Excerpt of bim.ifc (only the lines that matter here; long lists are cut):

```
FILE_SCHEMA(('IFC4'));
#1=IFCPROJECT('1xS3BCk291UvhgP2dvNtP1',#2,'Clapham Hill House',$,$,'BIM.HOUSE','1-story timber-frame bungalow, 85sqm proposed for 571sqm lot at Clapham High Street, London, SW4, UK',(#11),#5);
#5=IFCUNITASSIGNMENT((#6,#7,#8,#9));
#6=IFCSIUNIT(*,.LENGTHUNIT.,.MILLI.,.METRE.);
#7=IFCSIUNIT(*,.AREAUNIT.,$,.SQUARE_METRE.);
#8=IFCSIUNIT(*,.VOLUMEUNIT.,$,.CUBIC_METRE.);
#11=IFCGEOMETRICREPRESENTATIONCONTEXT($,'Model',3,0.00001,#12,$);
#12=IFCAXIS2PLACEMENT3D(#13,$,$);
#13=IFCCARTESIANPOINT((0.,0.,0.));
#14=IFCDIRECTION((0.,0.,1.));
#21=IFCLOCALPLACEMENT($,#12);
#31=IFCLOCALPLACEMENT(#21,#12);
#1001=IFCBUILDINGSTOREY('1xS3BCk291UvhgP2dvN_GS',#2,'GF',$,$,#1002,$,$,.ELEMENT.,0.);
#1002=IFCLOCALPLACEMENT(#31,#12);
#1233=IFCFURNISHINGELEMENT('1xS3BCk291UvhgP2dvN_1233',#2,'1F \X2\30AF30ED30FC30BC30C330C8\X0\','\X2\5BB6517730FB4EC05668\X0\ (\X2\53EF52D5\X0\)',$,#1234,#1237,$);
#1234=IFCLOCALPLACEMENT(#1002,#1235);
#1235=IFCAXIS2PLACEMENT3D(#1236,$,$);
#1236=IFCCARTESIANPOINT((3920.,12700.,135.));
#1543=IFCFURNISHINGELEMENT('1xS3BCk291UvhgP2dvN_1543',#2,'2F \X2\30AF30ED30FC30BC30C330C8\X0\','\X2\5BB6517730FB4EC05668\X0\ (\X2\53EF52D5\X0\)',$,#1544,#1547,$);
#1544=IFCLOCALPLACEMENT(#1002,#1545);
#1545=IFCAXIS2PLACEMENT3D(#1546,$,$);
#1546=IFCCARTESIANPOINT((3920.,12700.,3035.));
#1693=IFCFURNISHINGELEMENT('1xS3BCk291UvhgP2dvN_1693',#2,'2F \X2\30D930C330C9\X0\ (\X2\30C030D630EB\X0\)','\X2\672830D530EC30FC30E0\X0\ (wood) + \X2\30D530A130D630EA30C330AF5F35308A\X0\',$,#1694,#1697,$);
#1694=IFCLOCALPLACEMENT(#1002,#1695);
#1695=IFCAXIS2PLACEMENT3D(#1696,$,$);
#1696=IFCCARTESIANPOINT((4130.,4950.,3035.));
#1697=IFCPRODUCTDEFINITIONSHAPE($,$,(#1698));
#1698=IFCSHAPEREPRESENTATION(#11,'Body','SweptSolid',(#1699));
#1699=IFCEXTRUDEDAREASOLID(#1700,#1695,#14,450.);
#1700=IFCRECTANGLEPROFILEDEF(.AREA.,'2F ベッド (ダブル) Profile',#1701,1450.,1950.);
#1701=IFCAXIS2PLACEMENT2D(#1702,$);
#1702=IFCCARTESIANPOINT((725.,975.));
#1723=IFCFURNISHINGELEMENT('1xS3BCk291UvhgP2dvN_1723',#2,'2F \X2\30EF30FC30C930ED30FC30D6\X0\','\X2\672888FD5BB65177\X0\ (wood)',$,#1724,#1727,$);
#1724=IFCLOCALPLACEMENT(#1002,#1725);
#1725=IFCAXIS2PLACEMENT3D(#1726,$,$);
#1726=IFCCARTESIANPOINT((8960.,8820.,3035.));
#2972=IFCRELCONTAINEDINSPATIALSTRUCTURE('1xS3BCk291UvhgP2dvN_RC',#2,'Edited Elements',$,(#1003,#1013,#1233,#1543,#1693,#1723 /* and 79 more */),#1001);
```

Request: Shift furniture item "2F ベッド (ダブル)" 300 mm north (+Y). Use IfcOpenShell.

```python
import ifcopenshell
import ifcopenshell.api.geometry
import ifcopenshell.util.placement
import ifcopenshell.util.unit

model = ifcopenshell.open("bim.ifc")
unit_scale = ifcopenshell.util.unit.calculate_unit_scale(model)

item = model.by_id(1693)
matrix = ifcopenshell.util.placement.get_local_placement(item.ObjectPlacement)
matrix[1, 3] += 0.3 / unit_scale
ifcopenshell.api.geometry.edit_object_placement(model, product=item, matrix=matrix, is_si=False)

print(ifcopenshell.util.placement.get_local_placement(item.ObjectPlacement).round(3) + 0.0)

model.write("bim_rev.ifc")
```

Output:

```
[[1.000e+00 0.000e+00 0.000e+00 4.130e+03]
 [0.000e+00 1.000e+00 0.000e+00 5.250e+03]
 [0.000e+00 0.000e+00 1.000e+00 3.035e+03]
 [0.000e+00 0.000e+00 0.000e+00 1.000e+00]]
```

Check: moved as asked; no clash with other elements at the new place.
